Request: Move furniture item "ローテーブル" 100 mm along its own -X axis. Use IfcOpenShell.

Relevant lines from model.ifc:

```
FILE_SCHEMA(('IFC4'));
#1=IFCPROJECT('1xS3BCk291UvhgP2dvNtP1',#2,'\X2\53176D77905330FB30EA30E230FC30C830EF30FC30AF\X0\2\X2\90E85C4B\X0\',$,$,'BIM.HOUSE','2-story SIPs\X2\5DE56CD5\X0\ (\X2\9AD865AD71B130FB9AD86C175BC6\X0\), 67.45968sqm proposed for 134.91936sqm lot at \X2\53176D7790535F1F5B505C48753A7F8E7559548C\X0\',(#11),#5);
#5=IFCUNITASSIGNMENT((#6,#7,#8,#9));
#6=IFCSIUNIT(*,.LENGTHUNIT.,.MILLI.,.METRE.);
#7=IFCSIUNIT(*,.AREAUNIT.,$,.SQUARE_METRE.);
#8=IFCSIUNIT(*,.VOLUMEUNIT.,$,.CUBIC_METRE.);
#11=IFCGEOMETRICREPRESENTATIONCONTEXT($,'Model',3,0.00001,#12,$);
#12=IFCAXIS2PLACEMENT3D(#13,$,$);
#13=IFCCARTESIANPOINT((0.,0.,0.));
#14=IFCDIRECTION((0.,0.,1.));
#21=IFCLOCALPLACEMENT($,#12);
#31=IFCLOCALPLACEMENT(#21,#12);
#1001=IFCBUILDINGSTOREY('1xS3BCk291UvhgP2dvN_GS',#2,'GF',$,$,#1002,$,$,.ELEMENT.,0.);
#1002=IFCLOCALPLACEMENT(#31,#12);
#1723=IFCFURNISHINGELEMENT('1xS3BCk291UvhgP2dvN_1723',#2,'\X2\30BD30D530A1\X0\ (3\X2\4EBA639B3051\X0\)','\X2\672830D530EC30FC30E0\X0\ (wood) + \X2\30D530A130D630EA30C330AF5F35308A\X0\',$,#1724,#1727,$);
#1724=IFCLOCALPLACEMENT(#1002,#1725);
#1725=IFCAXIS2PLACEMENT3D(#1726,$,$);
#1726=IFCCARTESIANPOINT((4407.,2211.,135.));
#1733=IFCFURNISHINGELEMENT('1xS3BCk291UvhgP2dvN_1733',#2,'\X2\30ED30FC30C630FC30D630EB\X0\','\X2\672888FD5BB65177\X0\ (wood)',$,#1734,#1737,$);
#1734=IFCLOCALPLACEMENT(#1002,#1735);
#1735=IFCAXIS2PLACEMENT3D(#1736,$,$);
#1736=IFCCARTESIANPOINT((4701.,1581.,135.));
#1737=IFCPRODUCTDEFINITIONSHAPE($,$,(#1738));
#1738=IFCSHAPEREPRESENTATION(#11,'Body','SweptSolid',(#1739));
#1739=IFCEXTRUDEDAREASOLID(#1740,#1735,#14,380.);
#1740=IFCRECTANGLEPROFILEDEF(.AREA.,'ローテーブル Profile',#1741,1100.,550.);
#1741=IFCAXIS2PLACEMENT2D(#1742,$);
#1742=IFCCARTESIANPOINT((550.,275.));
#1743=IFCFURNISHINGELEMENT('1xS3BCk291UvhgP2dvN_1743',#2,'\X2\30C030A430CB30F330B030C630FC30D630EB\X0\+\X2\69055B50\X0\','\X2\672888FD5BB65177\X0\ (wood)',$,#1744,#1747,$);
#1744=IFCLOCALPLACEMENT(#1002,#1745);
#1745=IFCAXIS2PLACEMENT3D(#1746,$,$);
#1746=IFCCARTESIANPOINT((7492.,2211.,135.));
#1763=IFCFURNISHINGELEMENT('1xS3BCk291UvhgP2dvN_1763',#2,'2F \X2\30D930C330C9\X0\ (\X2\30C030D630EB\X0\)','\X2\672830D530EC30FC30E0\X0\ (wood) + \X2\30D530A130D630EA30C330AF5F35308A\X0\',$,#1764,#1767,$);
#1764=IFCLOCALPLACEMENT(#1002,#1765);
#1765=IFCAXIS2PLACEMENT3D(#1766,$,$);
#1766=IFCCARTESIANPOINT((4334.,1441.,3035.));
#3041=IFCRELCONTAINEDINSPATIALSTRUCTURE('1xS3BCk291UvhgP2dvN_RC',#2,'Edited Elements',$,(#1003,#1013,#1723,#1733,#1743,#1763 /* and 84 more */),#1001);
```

```python
import ifcopenshell
import ifcopenshell.api.geometry
import ifcopenshell.util.placement
import ifcopenshell.util.unit

model = ifcopenshell.open("model.ifc")
unit_scale = ifcopenshell.util.unit.calculate_unit_scale(model)

item = model.by_id(1733)
matrix = ifcopenshell.util.placement.get_local_placement(item.ObjectPlacement)
matrix[:3, 3] -= matrix[:3, 0] * 0.1 / unit_scale
ifcopenshell.api.geometry.edit_object_placement(model, product=item, matrix=matrix, is_si=False)

print(ifcopenshell.util.placement.get_local_placement(item.ObjectPlacement).round(3) + 0.0)

model.write("model_updated.ifc")
```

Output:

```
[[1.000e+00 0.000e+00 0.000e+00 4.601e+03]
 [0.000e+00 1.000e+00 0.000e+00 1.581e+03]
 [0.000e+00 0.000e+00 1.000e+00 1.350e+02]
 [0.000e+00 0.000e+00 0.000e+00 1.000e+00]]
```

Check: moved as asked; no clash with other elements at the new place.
